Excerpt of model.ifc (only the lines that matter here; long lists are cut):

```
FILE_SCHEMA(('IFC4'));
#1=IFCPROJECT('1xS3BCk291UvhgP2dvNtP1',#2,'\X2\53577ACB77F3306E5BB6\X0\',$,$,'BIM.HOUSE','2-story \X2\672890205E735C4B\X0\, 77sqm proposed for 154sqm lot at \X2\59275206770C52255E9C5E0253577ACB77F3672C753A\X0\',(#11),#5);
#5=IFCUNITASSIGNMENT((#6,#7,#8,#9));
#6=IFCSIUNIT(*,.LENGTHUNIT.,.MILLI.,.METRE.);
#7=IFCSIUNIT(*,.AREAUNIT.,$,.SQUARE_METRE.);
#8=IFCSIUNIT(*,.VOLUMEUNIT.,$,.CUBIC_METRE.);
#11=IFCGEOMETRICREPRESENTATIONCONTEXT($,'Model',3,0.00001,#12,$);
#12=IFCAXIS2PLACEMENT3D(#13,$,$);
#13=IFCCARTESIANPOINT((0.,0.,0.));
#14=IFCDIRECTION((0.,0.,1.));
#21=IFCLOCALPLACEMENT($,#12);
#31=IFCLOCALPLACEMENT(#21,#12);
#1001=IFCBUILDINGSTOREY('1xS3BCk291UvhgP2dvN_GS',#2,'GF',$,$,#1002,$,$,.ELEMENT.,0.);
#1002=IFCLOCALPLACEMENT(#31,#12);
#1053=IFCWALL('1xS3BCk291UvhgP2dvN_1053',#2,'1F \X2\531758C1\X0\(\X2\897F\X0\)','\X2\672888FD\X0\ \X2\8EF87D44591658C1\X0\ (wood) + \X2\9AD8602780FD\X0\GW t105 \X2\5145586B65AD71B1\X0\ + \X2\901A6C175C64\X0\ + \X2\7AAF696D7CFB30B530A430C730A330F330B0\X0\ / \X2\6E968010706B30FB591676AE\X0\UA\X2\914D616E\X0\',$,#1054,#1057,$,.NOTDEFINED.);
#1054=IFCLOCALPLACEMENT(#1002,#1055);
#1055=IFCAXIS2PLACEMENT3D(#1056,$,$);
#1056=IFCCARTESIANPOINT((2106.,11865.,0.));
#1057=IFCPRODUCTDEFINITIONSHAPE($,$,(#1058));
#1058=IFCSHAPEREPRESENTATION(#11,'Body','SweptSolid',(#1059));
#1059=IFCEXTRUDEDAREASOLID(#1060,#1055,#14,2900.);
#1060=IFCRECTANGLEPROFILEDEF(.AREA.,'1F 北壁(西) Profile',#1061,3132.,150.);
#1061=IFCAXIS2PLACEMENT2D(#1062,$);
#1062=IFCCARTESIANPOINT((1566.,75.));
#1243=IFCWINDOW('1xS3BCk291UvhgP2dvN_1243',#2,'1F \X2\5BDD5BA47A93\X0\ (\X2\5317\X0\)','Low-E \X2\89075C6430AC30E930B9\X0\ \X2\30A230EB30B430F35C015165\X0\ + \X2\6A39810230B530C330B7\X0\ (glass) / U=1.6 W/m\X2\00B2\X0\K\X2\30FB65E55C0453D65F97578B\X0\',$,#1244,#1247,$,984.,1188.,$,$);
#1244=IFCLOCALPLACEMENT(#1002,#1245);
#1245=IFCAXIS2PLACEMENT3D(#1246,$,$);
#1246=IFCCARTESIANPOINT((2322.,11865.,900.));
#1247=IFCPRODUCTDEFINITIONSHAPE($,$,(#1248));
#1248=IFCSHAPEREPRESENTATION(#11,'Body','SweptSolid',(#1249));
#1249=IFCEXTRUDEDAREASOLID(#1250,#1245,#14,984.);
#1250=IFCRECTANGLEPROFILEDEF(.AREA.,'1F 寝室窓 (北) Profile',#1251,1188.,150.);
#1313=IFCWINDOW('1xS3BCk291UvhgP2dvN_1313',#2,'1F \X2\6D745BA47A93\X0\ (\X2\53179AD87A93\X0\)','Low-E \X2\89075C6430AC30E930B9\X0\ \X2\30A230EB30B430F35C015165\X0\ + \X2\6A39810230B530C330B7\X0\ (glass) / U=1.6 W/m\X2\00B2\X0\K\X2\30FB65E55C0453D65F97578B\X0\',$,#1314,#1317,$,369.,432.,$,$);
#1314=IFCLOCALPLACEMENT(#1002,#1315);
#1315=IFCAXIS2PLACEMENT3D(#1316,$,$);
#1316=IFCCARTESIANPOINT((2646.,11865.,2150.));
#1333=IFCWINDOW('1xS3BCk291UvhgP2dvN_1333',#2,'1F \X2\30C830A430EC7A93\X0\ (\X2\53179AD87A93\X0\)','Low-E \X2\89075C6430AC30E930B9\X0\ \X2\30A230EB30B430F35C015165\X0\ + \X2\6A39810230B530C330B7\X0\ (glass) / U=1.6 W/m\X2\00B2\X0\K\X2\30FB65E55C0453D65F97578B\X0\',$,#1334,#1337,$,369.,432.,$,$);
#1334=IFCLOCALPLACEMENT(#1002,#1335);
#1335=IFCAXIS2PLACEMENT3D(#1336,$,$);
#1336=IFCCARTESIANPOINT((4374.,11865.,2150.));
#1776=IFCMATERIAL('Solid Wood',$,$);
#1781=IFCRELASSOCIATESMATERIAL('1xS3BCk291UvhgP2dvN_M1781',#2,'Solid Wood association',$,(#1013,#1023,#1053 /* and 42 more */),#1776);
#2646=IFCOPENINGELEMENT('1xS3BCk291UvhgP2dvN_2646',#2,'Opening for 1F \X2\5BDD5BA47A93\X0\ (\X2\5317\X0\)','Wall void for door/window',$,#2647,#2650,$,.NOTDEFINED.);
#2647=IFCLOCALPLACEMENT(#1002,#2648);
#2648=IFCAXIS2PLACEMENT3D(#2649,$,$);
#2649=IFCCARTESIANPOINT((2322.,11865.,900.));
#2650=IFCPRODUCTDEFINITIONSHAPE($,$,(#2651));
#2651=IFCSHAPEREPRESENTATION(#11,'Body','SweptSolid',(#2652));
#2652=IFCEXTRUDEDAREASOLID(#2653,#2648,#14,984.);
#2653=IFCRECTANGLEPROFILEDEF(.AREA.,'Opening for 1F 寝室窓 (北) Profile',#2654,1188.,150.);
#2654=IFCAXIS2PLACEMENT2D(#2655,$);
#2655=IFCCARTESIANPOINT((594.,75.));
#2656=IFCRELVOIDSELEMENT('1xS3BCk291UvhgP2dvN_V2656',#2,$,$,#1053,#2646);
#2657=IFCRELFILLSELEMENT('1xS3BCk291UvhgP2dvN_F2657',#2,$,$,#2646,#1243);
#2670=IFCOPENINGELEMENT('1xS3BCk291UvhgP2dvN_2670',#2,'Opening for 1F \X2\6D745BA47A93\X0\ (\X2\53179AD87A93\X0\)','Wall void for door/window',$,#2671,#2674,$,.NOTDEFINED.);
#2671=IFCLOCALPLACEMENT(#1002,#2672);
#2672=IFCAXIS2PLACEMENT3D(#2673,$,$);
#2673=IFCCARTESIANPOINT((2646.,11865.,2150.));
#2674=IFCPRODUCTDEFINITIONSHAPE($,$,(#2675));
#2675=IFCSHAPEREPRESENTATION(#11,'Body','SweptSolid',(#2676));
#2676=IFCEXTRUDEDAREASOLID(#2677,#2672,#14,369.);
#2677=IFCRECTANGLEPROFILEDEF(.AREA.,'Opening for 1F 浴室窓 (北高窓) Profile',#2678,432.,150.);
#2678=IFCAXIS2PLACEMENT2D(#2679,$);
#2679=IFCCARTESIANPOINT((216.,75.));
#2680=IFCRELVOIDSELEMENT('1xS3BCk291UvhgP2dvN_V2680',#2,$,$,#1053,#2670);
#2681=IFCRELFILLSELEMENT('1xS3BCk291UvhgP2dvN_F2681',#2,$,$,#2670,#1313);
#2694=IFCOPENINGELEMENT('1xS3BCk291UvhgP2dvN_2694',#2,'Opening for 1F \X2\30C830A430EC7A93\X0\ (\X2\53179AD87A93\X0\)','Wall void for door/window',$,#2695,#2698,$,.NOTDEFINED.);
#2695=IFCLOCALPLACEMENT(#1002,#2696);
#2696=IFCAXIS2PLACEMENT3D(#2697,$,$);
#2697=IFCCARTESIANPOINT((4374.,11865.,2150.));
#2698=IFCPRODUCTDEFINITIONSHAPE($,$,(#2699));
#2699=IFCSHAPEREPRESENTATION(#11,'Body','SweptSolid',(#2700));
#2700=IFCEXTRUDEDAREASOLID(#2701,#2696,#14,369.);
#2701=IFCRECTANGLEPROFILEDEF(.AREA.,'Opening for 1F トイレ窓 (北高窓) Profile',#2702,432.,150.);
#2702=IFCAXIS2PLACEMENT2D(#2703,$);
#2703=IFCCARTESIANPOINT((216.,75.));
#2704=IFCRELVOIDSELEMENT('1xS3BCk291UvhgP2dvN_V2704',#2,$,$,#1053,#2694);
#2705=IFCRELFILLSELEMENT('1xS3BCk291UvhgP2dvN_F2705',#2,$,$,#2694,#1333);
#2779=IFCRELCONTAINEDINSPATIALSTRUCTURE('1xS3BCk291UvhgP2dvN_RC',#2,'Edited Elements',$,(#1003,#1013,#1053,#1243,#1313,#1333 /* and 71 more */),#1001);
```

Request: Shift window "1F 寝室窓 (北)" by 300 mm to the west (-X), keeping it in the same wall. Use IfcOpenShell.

```python
import ifcopenshell
import ifcopenshell.api.geometry
import ifcopenshell.util.placement
import ifcopenshell.util.unit

model = ifcopenshell.open("model.ifc")
unit_scale = ifcopenshell.util.unit.calculate_unit_scale(model)

window = model.by_guid("1xS3BCk291UvhgP2dvN_1243")
opening = window.FillsVoids[0].RelatingOpeningElement
wall = opening.VoidsElements[0].RelatingBuildingElement

wall_matrix = ifcopenshell.util.placement.get_local_placement(wall.ObjectPlacement)
shift = wall_matrix[:3, 0] * -0.3 / unit_scale
before = ifcopenshell.util.placement.get_local_placement(window.ObjectPlacement)[:3, 3].copy()

# The window is not placed relative to its opening, so move both.
for product in (opening, window):
    matrix = ifcopenshell.util.placement.get_local_placement(product.ObjectPlacement)
    matrix[:3, 3] += shift
    ifcopenshell.api.geometry.edit_object_placement(model, product=product, matrix=matrix, is_si=False)

after = ifcopenshell.util.placement.get_local_placement(window.ObjectPlacement)[:3, 3]
print("window moved by", (after - before).round(3) + 0.0)

model.write("model-out.ifc")
```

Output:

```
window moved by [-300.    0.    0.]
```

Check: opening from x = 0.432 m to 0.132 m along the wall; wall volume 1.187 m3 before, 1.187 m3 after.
